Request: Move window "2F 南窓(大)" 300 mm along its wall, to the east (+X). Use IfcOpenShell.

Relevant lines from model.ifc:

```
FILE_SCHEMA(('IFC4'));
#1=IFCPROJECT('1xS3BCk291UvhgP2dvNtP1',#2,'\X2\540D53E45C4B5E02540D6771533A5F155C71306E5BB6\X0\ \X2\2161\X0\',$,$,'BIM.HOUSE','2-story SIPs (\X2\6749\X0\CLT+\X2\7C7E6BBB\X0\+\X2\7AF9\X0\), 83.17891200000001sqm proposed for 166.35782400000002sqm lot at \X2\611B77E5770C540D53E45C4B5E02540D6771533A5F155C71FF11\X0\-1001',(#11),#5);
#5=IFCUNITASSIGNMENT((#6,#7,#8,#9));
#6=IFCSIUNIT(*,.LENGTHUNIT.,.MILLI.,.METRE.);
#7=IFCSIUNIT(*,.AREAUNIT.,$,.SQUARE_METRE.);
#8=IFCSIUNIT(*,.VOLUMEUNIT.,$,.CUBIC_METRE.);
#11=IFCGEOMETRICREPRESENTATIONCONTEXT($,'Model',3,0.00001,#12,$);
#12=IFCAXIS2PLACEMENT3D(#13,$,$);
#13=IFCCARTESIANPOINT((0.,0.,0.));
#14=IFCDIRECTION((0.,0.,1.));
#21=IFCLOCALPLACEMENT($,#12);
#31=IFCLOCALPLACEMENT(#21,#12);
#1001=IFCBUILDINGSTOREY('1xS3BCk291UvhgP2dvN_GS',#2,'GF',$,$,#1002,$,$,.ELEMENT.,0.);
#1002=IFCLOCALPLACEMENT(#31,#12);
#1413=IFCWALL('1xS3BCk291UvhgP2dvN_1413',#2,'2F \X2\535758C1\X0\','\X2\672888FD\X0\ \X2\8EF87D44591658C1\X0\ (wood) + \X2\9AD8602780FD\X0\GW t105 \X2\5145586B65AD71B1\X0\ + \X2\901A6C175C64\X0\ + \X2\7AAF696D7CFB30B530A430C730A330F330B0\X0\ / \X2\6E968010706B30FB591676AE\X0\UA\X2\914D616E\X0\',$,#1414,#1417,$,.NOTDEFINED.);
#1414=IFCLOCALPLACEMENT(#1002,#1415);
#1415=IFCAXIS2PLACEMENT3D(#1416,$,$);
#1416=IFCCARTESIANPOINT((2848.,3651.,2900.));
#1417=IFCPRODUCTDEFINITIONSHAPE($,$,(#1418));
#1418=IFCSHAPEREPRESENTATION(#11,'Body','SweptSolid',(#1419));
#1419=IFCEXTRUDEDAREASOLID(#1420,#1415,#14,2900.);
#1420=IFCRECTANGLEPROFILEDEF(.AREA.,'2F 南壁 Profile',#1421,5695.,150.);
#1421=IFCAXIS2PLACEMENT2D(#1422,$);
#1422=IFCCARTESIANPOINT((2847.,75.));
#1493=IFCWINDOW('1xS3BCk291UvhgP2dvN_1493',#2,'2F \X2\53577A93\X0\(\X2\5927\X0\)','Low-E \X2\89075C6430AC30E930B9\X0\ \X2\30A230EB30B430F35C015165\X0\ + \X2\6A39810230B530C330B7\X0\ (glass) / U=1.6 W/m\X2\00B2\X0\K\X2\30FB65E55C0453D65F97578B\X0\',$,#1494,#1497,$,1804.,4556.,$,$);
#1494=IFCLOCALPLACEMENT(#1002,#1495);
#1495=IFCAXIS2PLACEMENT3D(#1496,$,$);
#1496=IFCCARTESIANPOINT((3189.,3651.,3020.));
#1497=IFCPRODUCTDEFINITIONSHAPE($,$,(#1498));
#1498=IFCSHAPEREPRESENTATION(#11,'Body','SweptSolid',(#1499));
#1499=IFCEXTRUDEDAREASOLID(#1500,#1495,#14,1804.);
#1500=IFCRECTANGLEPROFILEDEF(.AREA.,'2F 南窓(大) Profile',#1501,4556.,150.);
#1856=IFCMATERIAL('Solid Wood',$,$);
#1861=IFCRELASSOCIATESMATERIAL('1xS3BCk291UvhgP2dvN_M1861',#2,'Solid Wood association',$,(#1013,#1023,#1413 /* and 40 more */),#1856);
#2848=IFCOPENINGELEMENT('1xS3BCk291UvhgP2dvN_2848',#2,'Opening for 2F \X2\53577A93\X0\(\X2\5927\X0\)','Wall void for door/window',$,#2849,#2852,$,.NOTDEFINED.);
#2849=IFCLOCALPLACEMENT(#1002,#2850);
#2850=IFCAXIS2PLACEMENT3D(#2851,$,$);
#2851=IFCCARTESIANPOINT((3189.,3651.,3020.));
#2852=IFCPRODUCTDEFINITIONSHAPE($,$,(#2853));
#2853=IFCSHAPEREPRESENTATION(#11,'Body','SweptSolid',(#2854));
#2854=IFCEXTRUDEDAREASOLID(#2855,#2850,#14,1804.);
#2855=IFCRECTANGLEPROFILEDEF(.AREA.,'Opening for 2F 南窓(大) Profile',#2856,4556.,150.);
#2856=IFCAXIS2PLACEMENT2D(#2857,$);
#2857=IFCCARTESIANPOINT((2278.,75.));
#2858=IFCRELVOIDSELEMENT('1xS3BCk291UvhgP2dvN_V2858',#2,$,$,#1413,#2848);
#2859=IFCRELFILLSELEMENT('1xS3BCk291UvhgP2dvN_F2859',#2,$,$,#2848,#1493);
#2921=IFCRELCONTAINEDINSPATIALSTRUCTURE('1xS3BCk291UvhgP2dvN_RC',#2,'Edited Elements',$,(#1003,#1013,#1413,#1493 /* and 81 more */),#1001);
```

```python
import ifcopenshell
import ifcopenshell.api.geometry
import ifcopenshell.util.placement

model = ifcopenshell.open("model.ifc")

window = model.by_guid("1xS3BCk291UvhgP2dvN_1493")
opening = window.FillsVoids[0].RelatingOpeningElement
wall = opening.VoidsElements[0].RelatingBuildingElement

wall_matrix = ifcopenshell.util.placement.get_local_placement(wall.ObjectPlacement)
shift = wall_matrix[:3, 0] * 300.0
before = ifcopenshell.util.placement.get_local_placement(window.ObjectPlacement)[:3, 3].copy()

# The window is not placed relative to its opening, so move both.
for product in (opening, window):
    matrix = ifcopenshell.util.placement.get_local_placement(product.ObjectPlacement)
    matrix[:3, 3] += shift
    ifcopenshell.api.geometry.edit_object_placement(model, product=product, matrix=matrix, is_si=False)

after = ifcopenshell.util.placement.get_local_placement(window.ObjectPlacement)[:3, 3]
print("window moved by", (after - before).round(3) + 0.0)

model.write("model_v2.ifc")
```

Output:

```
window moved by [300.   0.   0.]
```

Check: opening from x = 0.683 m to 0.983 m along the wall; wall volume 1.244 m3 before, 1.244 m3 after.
